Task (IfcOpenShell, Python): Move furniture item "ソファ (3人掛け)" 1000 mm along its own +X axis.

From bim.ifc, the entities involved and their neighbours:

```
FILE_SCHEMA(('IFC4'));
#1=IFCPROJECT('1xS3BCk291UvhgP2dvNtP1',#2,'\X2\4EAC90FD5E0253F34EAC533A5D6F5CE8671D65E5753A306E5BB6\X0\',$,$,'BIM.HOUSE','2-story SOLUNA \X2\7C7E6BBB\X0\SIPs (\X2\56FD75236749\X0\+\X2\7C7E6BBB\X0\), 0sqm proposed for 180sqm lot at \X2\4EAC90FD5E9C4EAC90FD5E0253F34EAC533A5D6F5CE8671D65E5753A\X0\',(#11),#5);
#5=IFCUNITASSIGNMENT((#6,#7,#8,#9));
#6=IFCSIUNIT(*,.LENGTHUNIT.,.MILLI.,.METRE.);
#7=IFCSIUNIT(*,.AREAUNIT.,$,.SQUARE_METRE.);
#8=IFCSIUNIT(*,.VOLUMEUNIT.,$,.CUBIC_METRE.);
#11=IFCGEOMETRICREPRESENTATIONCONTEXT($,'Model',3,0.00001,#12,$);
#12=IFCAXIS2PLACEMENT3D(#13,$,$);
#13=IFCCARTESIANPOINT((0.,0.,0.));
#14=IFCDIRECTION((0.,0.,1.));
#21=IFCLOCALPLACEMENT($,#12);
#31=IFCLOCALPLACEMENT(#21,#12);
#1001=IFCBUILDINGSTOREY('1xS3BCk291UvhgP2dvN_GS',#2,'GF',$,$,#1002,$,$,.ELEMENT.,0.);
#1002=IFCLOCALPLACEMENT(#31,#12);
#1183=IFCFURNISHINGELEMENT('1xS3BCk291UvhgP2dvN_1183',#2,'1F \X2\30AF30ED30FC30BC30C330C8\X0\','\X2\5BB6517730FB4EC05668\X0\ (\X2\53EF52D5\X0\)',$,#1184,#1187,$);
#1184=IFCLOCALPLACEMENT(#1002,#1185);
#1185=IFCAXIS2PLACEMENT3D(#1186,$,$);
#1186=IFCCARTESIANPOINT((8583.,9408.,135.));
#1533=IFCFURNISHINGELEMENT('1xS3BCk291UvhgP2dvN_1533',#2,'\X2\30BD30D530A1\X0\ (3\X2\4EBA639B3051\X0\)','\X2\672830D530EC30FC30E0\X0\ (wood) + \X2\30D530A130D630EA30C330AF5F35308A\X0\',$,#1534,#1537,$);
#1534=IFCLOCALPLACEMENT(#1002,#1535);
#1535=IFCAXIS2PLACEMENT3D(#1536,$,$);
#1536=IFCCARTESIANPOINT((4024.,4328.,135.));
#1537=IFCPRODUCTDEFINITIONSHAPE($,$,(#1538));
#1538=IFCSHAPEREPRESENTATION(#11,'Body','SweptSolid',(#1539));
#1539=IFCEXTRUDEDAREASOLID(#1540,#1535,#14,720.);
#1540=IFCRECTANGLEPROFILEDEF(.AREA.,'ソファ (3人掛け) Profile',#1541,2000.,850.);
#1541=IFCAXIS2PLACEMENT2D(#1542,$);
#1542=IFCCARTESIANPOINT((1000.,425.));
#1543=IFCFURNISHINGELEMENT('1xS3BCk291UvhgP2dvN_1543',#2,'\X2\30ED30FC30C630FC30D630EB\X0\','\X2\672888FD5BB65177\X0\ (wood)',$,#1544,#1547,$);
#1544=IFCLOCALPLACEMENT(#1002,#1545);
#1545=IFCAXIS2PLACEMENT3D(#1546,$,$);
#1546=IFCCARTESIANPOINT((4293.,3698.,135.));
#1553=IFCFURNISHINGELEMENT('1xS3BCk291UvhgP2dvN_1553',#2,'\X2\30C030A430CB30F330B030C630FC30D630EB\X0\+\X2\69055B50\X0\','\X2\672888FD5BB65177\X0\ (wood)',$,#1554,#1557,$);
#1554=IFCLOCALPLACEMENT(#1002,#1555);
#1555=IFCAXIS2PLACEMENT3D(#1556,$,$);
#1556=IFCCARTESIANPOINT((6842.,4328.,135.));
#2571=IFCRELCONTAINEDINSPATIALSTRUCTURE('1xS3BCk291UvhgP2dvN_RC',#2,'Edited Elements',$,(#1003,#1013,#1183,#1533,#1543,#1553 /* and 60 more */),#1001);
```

```python
import ifcopenshell
import ifcopenshell.api.geometry
import ifcopenshell.util.placement
import ifcopenshell.util.unit

model = ifcopenshell.open("bim.ifc")
unit_scale = ifcopenshell.util.unit.calculate_unit_scale(model)

item = model.by_guid("1xS3BCk291UvhgP2dvN_1533")
matrix = ifcopenshell.util.placement.get_local_placement(item.ObjectPlacement)
matrix[:3, 3] += matrix[:3, 0] * 1 / unit_scale
ifcopenshell.api.geometry.edit_object_placement(model, product=item, matrix=matrix, is_si=False)

print(ifcopenshell.util.placement.get_local_placement(item.ObjectPlacement).round(3) + 0.0)

model.write("bim_rev.ifc")
```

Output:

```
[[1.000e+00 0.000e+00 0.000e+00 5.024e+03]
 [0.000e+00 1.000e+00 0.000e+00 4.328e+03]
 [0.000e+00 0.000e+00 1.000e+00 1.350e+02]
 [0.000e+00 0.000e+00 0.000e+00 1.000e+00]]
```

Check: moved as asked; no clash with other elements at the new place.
